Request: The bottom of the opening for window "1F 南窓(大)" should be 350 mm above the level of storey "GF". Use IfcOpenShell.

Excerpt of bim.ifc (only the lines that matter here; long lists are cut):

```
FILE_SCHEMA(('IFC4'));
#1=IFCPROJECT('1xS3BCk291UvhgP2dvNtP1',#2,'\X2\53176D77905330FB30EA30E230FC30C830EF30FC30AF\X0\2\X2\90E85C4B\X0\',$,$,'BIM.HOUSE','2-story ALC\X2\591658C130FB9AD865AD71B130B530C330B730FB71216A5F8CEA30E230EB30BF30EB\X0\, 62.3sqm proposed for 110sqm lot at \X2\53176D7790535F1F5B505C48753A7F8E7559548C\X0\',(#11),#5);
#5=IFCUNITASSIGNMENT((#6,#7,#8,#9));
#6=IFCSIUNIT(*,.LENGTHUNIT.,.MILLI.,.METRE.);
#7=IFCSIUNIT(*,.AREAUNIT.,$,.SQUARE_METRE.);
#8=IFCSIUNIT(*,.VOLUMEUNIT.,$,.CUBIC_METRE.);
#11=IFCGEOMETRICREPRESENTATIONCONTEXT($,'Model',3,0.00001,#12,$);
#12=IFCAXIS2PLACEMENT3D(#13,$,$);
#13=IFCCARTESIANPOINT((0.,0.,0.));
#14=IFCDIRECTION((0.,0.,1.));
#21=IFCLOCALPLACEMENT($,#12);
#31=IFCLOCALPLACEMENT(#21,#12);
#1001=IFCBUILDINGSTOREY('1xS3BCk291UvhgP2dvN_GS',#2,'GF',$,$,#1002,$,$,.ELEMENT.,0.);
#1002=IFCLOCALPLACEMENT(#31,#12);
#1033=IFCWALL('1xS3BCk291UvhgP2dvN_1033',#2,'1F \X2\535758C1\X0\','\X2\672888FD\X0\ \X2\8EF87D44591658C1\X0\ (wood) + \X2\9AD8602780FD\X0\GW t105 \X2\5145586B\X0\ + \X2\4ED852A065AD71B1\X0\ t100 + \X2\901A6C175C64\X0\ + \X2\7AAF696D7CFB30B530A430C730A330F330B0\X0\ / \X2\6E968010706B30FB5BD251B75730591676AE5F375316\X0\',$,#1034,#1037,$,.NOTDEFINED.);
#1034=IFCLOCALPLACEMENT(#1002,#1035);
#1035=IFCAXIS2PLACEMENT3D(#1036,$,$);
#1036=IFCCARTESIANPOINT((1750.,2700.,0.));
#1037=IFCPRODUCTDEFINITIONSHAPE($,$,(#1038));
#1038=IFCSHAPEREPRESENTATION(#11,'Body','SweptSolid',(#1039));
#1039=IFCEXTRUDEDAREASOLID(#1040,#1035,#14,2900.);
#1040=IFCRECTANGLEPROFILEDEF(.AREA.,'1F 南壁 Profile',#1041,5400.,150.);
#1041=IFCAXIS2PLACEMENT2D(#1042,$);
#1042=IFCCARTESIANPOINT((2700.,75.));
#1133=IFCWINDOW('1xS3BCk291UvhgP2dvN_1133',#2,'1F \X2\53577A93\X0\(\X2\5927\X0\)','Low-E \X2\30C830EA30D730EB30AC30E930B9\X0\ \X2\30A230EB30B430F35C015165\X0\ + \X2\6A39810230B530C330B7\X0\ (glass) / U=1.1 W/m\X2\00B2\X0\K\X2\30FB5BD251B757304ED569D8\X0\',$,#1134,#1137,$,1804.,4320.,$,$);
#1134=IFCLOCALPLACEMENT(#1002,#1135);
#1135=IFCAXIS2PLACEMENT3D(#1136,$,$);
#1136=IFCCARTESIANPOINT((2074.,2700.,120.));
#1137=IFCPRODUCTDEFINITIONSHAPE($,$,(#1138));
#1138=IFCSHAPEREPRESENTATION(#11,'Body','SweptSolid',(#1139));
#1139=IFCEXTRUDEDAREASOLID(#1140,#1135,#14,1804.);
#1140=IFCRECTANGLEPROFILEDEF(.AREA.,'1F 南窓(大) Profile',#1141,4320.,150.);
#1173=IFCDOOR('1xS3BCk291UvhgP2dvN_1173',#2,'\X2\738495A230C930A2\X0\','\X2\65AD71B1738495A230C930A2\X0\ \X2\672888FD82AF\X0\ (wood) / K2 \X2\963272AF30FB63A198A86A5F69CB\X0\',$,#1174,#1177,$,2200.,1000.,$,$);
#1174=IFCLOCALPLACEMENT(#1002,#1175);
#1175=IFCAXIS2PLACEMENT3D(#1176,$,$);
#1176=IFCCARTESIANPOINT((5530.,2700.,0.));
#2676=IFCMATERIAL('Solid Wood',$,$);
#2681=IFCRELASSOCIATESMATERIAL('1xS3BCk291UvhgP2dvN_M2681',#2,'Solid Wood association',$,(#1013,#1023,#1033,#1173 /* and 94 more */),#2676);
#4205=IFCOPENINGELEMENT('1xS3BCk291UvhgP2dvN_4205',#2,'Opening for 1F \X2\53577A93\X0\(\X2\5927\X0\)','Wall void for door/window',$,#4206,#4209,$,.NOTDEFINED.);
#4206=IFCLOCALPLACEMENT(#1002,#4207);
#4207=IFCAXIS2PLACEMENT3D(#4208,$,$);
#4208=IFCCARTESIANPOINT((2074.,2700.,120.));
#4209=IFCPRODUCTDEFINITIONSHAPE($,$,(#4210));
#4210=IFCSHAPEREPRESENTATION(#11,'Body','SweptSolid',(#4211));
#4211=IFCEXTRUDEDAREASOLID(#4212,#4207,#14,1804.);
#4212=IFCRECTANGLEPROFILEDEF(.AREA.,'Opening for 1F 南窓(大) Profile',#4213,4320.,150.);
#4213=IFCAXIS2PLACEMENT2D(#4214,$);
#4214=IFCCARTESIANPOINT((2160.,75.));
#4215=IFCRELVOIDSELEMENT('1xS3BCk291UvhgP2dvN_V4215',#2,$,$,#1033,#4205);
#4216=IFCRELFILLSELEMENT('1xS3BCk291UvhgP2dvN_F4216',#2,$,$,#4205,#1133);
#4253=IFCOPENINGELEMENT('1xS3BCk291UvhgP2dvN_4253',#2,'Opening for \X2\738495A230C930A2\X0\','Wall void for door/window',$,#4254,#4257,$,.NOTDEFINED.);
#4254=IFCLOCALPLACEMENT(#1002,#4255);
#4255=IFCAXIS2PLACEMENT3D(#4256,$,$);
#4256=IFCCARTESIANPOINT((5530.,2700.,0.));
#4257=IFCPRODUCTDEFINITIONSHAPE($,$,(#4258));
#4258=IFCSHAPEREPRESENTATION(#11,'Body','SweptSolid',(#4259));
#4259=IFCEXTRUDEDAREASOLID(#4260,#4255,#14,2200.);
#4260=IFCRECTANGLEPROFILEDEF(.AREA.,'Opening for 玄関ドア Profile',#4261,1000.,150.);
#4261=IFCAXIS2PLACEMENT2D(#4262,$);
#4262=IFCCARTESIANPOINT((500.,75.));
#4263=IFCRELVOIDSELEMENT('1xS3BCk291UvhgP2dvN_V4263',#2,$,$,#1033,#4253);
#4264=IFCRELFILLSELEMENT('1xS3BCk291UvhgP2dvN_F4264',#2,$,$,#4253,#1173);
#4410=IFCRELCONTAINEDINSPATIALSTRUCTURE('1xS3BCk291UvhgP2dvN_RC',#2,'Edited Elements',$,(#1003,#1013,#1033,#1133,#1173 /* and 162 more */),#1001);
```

```python
import numpy as np
import ifcopenshell
import ifcopenshell.api.geometry
import ifcopenshell.geom
import ifcopenshell.util.element
import ifcopenshell.util.placement
import ifcopenshell.util.shape
import ifcopenshell.util.unit

model = ifcopenshell.open("bim.ifc")
unit_scale = ifcopenshell.util.unit.calculate_unit_scale(model)

window = model.by_guid("1xS3BCk291UvhgP2dvN_1133")
opening = window.FillsVoids[0].RelatingOpeningElement
storey = ifcopenshell.util.element.get_container(window, ifc_class="IfcBuildingStorey")
level = ifcopenshell.util.placement.get_local_placement(storey.ObjectPlacement)[2, 3]

# The opening's origin need not be at the sill, so measure its lowest point.
shape = ifcopenshell.geom.create_shape(ifcopenshell.geom.settings(), opening)
bottom = ifcopenshell.util.shape.get_shape_bottom_elevation(shape, shape.geometry) / unit_scale
dz = level + 0.35 / unit_scale - bottom

shift = np.array([0.0, 0.0, dz])
# The window is not placed relative to its opening, so move both.
for product in (opening, window):
    matrix = ifcopenshell.util.placement.get_local_placement(product.ObjectPlacement)
    matrix[:3, 3] += shift
    ifcopenshell.api.geometry.edit_object_placement(model, product=product, matrix=matrix, is_si=False)

print(f"moved by {dz * unit_scale:+.3f} m")

model.write("bim_updated.ifc")
```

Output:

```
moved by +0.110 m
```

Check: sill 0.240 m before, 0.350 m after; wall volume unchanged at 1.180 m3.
